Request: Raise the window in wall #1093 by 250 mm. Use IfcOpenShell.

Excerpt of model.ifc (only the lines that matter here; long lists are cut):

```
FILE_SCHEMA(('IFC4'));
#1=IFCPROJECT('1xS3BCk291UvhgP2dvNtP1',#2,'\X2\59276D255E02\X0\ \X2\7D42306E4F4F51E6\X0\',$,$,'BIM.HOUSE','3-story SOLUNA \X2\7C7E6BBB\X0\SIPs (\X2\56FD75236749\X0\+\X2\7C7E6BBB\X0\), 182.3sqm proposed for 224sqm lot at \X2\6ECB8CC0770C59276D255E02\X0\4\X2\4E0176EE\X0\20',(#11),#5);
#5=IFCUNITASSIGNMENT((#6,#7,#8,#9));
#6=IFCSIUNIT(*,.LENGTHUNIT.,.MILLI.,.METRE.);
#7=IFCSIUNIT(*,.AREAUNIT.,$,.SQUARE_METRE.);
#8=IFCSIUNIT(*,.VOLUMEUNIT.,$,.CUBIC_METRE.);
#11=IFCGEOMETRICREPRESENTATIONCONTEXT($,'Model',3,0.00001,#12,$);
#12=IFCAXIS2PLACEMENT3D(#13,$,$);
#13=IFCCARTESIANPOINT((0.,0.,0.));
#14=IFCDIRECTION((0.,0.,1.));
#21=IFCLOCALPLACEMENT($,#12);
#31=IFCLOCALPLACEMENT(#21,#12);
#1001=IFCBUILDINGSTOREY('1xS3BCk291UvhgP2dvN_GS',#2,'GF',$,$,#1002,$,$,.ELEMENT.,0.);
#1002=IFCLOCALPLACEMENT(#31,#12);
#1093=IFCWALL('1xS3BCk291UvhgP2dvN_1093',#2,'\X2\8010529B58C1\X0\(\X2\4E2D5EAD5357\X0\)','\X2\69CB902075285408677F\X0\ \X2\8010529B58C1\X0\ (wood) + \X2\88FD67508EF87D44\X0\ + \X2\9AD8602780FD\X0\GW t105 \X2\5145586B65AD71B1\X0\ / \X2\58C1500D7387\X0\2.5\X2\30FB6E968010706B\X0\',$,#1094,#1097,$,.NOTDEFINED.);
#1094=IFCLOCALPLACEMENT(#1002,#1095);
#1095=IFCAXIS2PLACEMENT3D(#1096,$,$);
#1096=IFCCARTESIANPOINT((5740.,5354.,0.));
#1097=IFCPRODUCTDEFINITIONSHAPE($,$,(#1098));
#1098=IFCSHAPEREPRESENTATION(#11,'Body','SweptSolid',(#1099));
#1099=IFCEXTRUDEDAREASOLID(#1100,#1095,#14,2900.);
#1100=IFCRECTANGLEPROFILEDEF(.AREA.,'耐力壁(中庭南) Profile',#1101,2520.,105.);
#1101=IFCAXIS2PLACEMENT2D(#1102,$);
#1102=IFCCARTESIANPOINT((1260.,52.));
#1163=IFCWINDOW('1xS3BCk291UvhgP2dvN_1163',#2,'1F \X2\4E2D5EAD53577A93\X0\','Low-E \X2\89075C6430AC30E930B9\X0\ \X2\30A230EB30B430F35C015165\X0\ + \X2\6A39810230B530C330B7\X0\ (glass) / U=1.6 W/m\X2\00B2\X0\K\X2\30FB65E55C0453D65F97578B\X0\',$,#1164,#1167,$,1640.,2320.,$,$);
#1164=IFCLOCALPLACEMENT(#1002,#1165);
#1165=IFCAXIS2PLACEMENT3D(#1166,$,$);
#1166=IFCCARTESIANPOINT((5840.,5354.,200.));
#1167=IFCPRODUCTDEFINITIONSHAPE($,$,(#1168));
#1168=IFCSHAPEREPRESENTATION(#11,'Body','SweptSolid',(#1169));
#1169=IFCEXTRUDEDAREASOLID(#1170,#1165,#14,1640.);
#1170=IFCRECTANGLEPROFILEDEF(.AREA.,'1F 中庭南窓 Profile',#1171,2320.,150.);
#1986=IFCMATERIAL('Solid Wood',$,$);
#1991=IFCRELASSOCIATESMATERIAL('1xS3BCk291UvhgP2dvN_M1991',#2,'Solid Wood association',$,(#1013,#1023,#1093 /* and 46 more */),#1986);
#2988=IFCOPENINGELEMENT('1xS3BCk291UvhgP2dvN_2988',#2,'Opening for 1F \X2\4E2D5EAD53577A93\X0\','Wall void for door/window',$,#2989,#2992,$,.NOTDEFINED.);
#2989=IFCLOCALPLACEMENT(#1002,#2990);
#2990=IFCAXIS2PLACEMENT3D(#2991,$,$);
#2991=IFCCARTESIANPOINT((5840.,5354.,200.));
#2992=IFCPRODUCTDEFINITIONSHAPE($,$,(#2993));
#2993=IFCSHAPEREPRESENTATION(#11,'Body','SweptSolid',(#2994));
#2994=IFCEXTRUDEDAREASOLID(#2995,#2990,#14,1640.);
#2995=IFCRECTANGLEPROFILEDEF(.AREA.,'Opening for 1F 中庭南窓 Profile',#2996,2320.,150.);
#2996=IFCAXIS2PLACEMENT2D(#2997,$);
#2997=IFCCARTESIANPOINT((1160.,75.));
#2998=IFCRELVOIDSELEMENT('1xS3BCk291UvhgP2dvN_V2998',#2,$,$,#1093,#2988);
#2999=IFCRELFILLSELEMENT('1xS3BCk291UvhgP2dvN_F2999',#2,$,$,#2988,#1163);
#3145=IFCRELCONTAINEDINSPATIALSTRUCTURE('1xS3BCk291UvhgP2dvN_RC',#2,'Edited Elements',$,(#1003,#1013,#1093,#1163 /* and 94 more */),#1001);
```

```python
import numpy as np
import ifcopenshell
import ifcopenshell.api.geometry
import ifcopenshell.util.placement
import ifcopenshell.util.unit

model = ifcopenshell.open("model.ifc")
unit_scale = ifcopenshell.util.unit.calculate_unit_scale(model)

window = model.by_id(1163)
opening = window.FillsVoids[0].RelatingOpeningElement
dz = 0.25 / unit_scale

shift = np.array([0.0, 0.0, dz])
# The window is not placed relative to its opening, so move both.
for product in (opening, window):
    matrix = ifcopenshell.util.placement.get_local_placement(product.ObjectPlacement)
    matrix[:3, 3] += shift
    ifcopenshell.api.geometry.edit_object_placement(model, product=product, matrix=matrix, is_si=False)

print(f"moved by {dz * unit_scale:+.3f} m")

model.write("model_v2.ifc")
```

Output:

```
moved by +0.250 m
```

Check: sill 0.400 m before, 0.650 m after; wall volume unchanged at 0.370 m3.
